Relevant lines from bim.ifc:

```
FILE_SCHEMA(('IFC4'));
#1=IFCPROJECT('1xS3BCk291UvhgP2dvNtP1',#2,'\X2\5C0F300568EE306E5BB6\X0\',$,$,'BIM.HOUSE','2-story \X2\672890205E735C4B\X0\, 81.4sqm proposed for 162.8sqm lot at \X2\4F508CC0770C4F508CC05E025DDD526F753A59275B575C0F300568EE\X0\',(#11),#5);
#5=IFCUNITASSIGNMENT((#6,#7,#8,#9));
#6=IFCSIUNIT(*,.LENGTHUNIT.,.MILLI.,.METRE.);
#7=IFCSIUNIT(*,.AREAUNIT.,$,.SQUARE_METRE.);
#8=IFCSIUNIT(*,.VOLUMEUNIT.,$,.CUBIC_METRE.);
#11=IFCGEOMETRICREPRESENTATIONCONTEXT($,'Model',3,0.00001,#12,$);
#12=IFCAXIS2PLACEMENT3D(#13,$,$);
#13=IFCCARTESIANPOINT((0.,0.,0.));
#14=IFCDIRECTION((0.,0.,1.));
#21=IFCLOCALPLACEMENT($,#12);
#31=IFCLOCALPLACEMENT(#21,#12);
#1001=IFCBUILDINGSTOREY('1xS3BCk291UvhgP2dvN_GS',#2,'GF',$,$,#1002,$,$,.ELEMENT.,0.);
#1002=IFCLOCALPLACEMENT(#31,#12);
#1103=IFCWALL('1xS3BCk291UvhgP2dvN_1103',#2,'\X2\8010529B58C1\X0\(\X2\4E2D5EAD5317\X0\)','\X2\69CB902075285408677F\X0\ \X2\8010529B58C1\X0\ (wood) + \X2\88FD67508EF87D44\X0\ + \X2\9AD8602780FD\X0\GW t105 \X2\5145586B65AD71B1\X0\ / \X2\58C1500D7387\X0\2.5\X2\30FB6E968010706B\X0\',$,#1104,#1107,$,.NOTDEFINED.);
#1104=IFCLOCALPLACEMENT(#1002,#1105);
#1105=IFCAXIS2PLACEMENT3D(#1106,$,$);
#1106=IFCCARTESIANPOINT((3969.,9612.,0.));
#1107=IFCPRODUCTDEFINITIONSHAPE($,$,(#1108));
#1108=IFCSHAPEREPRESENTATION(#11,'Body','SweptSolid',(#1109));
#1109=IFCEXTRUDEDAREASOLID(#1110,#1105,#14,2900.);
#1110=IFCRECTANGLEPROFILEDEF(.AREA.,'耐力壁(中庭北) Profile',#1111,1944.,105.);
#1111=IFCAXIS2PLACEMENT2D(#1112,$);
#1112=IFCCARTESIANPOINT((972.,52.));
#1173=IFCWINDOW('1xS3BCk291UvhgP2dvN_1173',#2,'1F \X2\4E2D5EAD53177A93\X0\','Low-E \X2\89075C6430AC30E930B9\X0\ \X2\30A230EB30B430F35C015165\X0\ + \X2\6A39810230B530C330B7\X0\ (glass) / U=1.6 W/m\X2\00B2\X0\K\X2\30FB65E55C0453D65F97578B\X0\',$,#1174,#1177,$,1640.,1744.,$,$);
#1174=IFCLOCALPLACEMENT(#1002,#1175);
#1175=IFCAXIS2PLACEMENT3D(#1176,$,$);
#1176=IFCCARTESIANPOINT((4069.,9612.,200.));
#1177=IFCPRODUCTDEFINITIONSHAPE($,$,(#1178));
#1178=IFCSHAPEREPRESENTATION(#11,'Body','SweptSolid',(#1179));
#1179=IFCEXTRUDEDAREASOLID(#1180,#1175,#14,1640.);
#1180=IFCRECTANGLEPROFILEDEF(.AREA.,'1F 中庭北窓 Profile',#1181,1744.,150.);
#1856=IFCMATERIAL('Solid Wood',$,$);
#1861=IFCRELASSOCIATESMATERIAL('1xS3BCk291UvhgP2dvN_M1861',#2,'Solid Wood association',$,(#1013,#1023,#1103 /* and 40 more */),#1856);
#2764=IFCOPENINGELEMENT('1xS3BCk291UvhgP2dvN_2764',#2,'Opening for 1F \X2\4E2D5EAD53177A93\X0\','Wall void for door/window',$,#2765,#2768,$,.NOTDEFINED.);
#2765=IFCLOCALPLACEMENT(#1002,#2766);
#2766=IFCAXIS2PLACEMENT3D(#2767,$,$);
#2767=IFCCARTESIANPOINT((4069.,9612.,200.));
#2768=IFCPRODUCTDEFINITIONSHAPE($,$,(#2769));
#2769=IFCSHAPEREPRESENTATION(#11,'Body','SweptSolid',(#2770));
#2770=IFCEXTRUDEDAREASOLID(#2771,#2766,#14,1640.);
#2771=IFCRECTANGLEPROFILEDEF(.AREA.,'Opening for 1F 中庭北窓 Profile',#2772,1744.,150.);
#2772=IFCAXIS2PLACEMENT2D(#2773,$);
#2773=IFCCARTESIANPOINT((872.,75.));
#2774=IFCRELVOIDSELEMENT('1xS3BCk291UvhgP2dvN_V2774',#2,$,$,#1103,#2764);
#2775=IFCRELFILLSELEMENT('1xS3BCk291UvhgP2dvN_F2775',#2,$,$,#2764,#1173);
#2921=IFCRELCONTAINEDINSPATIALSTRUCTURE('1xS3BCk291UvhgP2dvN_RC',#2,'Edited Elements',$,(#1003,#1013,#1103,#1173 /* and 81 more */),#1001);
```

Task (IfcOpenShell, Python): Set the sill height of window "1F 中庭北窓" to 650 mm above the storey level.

```python
import numpy as np
import ifcopenshell
import ifcopenshell.api.geometry
import ifcopenshell.geom
import ifcopenshell.util.element
import ifcopenshell.util.placement
import ifcopenshell.util.shape
import ifcopenshell.util.unit

model = ifcopenshell.open("bim.ifc")
unit_scale = ifcopenshell.util.unit.calculate_unit_scale(model)

window = model.by_id(1173)
opening = window.FillsVoids[0].RelatingOpeningElement
storey = ifcopenshell.util.element.get_container(window, ifc_class="IfcBuildingStorey")
level = ifcopenshell.util.placement.get_local_placement(storey.ObjectPlacement)[2, 3]

# The opening's origin need not be at the sill, so measure its lowest point.
shape = ifcopenshell.geom.create_shape(ifcopenshell.geom.settings(), opening)
bottom = ifcopenshell.util.shape.get_shape_bottom_elevation(shape, shape.geometry) / unit_scale
dz = level + 0.65 / unit_scale - bottom

shift = np.array([0.0, 0.0, dz])
# The window is not placed relative to its opening, so move both.
for product in (opening, window):
    matrix = ifcopenshell.util.placement.get_local_placement(product.ObjectPlacement)
    matrix[:3, 3] += shift
    ifcopenshell.api.geometry.edit_object_placement(model, product=product, matrix=matrix, is_si=False)

print(f"moved by {dz * unit_scale:+.3f} m")

model.write("bim-out.ifc")
```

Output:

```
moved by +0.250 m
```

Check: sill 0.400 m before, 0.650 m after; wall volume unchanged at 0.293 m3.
